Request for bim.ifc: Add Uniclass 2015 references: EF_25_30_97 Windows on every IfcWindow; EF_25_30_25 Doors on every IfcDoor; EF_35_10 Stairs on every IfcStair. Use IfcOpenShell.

First a look at what the model holds.

```python
import ifcopenshell

model = ifcopenshell.open("bim.ifc")
print(model.schema)
print("classifications:", [c.Name for c in model.by_type("IfcClassification")])
for ifc_class in ("IfcDoor", "IfcRoof", "IfcStair", "IfcWall", "IfcWindow"):
    print(ifc_class, len(model.by_type(ifc_class)))
```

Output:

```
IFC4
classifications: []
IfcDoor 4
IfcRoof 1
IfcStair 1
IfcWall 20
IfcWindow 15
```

```python
import ifcopenshell
import ifcopenshell.api.classification

model = ifcopenshell.open("bim.ifc")

system = ifcopenshell.api.classification.add_classification(model, classification="Uniclass 2015")

codes = {
    "IfcWindow": ("EF_25_30_97", "Windows"),
    "IfcDoor": ("EF_25_30_25", "Doors"),
    "IfcStair": ("EF_35_10", "Stairs"),
}
for ifc_class, (code, name) in codes.items():
    products = model.by_type(ifc_class)
    ifcopenshell.api.classification.add_reference(
        model, products=products, classification=system, identification=code, name=name
    )
    print(code, len(products))

model.write("bim_updated.ifc")
```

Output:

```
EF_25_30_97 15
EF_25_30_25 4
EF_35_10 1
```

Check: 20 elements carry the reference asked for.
